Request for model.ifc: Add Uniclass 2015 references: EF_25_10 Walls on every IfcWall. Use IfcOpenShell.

First a look at what the model holds.

```python
import ifcopenshell

model = ifcopenshell.open("model.ifc")
print(model.schema)
print("classifications:", [c.Name for c in model.by_type("IfcClassification")])
for ifc_class in ("IfcDoor", "IfcRoof", "IfcStair", "IfcWall", "IfcWindow"):
    print(ifc_class, len(model.by_type(ifc_class)))
```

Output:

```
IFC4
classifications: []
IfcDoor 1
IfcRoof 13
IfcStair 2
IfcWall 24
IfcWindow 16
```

```python
import ifcopenshell
import ifcopenshell.api.classification

model = ifcopenshell.open("model.ifc")

system = ifcopenshell.api.classification.add_classification(model, classification="Uniclass 2015")

codes = {
    "IfcWall": ("EF_25_10", "Walls"),
}
for ifc_class, (code, name) in codes.items():
    products = model.by_type(ifc_class)
    ifcopenshell.api.classification.add_reference(
        model, products=products, classification=system, identification=code, name=name
    )
    print(code, len(products))

model.write("model-out.ifc")
```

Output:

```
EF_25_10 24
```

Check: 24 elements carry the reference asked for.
